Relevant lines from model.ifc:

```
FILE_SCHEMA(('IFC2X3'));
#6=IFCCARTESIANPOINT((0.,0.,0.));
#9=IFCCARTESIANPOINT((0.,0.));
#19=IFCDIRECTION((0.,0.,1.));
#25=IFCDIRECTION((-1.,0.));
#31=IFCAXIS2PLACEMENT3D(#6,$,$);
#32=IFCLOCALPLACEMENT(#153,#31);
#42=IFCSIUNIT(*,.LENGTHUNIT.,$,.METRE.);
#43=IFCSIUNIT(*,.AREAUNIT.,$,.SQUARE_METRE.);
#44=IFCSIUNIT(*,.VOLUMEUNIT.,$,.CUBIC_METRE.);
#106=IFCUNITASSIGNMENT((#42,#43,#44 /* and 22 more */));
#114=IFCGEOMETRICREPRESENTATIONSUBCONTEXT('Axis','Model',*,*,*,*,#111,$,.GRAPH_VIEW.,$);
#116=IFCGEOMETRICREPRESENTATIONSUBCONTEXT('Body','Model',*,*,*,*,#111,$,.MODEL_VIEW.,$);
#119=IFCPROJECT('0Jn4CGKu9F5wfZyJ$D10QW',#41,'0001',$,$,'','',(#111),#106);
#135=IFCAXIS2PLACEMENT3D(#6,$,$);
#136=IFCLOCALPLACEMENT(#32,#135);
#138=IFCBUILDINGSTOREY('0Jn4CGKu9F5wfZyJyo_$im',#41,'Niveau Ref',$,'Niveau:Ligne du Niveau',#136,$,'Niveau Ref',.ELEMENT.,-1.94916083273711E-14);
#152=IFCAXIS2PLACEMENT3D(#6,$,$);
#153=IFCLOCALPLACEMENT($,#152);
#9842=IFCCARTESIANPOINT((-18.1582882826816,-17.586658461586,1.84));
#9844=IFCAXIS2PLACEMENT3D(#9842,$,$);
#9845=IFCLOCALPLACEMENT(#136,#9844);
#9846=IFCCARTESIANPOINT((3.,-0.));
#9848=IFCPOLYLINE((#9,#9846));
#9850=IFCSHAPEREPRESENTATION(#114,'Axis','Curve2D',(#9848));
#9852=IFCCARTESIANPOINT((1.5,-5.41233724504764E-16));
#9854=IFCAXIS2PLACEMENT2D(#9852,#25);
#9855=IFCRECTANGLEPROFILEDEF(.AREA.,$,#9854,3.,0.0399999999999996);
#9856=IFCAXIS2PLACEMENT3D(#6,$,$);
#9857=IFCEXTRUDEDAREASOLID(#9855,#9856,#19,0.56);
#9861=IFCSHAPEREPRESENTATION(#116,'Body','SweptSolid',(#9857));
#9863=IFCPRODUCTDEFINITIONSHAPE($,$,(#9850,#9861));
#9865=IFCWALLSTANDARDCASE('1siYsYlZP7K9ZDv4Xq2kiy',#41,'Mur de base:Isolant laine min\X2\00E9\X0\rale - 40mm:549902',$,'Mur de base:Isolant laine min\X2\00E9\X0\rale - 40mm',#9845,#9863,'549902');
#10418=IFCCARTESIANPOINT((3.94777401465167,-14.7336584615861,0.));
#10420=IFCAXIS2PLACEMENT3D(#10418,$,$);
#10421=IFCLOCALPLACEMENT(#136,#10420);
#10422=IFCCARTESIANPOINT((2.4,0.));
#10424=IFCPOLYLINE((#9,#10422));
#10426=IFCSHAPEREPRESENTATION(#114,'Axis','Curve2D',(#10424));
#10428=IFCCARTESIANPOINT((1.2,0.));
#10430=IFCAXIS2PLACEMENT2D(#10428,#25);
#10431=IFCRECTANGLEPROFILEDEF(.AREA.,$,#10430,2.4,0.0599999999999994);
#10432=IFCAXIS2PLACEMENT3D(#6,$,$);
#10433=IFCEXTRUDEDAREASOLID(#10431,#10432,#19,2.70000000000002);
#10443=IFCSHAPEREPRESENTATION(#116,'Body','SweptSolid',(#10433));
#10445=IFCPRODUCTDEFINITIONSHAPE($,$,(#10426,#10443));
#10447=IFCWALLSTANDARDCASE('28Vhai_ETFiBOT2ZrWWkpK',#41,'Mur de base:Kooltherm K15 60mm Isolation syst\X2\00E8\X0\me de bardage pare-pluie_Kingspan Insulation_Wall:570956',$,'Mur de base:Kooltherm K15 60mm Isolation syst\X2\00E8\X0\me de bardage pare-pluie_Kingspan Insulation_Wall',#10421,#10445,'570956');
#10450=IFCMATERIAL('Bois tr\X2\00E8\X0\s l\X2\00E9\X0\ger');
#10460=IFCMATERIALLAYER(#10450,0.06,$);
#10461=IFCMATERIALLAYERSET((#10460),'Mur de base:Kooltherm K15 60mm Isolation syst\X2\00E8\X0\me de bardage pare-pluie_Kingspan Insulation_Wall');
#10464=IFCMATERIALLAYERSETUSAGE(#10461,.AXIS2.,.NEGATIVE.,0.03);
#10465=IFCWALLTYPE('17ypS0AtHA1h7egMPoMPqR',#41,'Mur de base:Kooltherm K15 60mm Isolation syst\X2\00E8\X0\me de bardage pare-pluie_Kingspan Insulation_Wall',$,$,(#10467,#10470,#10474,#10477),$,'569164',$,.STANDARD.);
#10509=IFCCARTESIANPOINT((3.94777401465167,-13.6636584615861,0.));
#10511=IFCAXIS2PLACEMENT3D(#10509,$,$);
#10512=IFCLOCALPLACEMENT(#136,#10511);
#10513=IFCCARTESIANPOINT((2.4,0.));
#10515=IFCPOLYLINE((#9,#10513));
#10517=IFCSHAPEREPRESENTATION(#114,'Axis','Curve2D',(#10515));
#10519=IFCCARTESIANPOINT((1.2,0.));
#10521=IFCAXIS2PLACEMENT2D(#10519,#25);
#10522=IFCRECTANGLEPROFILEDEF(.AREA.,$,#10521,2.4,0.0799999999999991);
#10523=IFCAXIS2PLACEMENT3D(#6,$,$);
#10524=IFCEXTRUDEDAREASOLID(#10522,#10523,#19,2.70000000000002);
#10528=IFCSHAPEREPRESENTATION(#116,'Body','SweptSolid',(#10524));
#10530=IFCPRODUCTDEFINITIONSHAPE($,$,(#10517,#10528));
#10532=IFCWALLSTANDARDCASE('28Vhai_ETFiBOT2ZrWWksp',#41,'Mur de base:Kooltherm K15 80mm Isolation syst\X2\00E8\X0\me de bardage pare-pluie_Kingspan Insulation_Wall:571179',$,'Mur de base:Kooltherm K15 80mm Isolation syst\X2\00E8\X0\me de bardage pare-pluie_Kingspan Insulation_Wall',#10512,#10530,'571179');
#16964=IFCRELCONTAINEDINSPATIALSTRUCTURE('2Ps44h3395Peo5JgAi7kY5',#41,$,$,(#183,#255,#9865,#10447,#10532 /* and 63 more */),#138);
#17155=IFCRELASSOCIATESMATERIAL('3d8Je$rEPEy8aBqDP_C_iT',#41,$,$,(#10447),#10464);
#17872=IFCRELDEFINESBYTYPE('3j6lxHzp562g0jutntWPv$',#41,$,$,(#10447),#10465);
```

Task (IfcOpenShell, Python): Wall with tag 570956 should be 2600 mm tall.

```python
import ifcopenshell
import ifcopenshell.geom
import ifcopenshell.util.representation
import ifcopenshell.util.shape
import ifcopenshell.util.unit

model = ifcopenshell.open("model.ifc")
unit_scale = ifcopenshell.util.unit.calculate_unit_scale(model)
settings = ifcopenshell.geom.settings()


def volume(element):
    """Net volume in cubic metres, openings subtracted."""
    shape = ifcopenshell.geom.create_shape(settings, element)
    return ifcopenshell.util.shape.get_volume(shape.geometry)


wall = model.by_guid("28Vhai_ETFiBOT2ZrWWkpK")
before = volume(wall)

body = ifcopenshell.util.representation.get_representation(wall, "Model", "Body")
solid = body.Items[0]
old_height = solid.Depth
solid.Depth = 2.6 / unit_scale
after = volume(wall)

print(f"height {old_height:g} -> {solid.Depth:g}, volume {before:.3f} -> {after:.3f} m3")

model.write("model_edited.ifc")
```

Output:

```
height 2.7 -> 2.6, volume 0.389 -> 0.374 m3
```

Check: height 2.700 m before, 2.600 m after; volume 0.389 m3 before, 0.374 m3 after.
